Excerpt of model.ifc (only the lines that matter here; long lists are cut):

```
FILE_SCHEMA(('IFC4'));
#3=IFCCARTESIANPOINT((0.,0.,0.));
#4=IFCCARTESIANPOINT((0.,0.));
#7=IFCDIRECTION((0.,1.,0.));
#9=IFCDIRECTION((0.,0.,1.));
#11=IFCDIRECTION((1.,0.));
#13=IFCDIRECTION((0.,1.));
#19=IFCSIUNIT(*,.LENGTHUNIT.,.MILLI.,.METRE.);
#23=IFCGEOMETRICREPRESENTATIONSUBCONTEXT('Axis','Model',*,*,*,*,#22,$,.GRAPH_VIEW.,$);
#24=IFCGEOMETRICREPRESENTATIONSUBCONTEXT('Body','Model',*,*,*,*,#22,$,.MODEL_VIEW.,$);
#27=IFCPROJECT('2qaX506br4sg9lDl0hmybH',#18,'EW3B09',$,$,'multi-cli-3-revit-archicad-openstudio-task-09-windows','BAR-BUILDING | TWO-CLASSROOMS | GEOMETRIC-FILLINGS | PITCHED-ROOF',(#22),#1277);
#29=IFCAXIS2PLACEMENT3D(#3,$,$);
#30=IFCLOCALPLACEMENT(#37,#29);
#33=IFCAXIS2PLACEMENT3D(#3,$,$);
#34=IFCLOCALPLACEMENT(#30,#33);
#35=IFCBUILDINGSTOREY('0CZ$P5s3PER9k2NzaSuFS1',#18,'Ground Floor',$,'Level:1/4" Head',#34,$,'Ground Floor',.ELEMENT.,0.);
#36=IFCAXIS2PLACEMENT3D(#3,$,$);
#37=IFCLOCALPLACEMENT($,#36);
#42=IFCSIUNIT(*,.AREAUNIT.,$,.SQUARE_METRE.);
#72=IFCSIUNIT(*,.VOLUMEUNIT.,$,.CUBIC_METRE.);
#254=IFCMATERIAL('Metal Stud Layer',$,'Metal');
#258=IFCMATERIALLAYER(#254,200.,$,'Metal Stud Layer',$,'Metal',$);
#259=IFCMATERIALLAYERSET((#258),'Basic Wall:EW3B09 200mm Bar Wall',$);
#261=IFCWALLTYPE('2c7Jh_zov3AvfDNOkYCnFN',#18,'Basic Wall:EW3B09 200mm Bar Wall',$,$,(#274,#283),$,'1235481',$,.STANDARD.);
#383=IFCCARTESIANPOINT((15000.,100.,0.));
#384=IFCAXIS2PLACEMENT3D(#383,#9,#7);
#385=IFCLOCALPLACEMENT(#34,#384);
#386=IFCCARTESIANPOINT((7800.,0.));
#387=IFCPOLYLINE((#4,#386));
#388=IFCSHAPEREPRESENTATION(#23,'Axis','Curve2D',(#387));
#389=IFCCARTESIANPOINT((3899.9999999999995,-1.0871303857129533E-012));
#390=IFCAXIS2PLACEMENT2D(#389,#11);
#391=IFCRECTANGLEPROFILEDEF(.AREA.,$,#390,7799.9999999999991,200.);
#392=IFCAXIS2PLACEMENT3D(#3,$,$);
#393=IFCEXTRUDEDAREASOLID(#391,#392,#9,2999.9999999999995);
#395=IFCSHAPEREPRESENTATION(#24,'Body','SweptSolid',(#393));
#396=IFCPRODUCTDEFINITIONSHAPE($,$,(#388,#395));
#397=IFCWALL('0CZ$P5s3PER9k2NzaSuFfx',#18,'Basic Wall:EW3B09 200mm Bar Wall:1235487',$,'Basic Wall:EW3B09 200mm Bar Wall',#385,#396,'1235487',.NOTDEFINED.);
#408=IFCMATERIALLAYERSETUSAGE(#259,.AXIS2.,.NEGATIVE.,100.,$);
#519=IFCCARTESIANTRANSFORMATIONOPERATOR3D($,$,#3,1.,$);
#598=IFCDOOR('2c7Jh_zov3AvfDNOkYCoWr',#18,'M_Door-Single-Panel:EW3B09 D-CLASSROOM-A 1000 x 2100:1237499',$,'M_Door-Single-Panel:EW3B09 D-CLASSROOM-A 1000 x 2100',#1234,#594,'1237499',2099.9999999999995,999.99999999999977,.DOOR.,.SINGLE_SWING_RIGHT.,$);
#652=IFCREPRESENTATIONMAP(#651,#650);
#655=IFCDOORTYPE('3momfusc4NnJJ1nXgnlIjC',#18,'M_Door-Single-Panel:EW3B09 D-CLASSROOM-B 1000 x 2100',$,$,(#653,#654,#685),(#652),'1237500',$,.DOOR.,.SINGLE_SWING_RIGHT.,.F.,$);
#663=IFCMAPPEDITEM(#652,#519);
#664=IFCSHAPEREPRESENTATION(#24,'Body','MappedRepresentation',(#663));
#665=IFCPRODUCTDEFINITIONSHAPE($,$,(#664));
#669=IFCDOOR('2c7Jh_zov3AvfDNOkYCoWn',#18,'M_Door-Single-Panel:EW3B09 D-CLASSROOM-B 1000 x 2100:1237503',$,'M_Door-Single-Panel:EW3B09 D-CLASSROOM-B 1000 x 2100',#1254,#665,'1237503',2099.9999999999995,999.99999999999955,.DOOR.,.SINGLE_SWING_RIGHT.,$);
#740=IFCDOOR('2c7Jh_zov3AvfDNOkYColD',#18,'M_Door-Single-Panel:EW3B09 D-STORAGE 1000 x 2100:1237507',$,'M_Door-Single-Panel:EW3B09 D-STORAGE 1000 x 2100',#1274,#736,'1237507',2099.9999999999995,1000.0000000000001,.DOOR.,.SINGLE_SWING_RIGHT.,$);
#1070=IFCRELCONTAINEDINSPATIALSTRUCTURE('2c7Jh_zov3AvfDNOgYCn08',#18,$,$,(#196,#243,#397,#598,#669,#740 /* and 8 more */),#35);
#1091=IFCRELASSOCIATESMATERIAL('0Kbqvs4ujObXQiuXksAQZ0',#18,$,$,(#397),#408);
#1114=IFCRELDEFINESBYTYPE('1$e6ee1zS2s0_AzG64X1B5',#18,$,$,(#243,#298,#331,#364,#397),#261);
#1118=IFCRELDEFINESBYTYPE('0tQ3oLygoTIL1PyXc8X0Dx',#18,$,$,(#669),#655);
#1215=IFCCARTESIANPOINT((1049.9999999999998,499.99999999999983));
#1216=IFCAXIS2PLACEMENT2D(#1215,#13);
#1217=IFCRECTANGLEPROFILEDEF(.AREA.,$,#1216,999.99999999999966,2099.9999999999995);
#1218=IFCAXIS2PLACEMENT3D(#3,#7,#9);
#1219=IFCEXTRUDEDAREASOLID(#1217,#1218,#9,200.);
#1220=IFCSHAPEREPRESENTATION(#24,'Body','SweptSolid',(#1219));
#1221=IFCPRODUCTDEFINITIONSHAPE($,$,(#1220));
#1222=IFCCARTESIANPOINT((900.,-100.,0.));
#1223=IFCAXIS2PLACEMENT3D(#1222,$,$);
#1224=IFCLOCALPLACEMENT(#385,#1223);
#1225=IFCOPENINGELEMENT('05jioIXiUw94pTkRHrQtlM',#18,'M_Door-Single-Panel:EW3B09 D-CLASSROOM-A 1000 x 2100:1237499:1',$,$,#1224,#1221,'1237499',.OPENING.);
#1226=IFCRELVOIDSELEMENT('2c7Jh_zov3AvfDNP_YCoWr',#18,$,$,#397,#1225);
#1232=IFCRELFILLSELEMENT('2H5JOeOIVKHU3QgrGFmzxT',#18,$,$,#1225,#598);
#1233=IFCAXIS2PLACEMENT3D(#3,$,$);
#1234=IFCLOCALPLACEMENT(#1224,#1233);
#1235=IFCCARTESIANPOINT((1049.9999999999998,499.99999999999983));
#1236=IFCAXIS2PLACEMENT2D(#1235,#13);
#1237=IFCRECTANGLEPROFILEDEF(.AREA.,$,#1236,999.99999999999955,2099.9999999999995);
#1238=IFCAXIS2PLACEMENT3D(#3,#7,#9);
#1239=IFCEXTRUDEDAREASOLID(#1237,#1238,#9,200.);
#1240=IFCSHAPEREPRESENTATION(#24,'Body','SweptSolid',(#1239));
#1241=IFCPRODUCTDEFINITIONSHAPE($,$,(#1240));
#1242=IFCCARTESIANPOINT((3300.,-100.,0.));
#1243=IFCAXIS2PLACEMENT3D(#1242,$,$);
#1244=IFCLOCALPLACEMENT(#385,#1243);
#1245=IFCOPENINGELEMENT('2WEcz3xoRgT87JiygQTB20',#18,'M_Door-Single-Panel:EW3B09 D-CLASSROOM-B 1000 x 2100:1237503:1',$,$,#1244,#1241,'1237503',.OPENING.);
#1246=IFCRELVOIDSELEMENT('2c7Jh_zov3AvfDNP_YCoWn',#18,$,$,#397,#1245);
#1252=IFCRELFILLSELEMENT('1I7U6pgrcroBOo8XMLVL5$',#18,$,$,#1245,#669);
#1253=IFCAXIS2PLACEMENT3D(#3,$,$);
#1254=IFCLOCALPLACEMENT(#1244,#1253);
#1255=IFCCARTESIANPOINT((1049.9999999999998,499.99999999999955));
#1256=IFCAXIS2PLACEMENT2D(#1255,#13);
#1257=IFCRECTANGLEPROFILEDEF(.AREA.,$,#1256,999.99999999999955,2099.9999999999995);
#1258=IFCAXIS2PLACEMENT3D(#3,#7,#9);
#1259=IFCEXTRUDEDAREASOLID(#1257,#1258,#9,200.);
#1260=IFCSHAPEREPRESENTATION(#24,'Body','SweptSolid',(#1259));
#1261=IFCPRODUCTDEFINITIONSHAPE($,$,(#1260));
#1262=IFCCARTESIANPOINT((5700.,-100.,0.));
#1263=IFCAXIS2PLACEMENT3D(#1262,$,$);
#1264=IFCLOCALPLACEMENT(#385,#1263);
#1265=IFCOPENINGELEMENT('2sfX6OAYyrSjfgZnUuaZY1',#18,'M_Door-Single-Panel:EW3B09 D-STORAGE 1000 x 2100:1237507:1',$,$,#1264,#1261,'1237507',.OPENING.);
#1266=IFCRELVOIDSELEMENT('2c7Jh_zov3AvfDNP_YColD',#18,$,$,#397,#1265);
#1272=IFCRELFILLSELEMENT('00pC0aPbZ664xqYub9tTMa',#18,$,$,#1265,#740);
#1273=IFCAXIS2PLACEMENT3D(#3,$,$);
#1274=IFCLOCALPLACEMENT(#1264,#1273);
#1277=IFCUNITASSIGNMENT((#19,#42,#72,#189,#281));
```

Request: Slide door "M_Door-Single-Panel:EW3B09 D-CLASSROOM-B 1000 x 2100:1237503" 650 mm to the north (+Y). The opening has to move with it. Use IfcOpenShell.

```python
import ifcopenshell
import ifcopenshell.api.geometry
import ifcopenshell.util.placement

model = ifcopenshell.open("model.ifc")

door = model.by_id(669)
opening = door.FillsVoids[0].RelatingOpeningElement
wall = opening.VoidsElements[0].RelatingBuildingElement

wall_matrix = ifcopenshell.util.placement.get_local_placement(wall.ObjectPlacement)
shift = wall_matrix[:3, 0] * 650.0
before = ifcopenshell.util.placement.get_local_placement(door.ObjectPlacement)[:3, 3].copy()

# The door is placed relative to its opening, so it follows when the opening moves.
matrix = ifcopenshell.util.placement.get_local_placement(opening.ObjectPlacement)
matrix[:3, 3] += shift
ifcopenshell.api.geometry.edit_object_placement(
    model, product=opening, matrix=matrix, is_si=False, should_transform_children=True
)

after = ifcopenshell.util.placement.get_local_placement(door.ObjectPlacement)[:3, 3]
print("door moved by", (after - before).round(3) + 0.0)

model.write("model-out.ifc")
```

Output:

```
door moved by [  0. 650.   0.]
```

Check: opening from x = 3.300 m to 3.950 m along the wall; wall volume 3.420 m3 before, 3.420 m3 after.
